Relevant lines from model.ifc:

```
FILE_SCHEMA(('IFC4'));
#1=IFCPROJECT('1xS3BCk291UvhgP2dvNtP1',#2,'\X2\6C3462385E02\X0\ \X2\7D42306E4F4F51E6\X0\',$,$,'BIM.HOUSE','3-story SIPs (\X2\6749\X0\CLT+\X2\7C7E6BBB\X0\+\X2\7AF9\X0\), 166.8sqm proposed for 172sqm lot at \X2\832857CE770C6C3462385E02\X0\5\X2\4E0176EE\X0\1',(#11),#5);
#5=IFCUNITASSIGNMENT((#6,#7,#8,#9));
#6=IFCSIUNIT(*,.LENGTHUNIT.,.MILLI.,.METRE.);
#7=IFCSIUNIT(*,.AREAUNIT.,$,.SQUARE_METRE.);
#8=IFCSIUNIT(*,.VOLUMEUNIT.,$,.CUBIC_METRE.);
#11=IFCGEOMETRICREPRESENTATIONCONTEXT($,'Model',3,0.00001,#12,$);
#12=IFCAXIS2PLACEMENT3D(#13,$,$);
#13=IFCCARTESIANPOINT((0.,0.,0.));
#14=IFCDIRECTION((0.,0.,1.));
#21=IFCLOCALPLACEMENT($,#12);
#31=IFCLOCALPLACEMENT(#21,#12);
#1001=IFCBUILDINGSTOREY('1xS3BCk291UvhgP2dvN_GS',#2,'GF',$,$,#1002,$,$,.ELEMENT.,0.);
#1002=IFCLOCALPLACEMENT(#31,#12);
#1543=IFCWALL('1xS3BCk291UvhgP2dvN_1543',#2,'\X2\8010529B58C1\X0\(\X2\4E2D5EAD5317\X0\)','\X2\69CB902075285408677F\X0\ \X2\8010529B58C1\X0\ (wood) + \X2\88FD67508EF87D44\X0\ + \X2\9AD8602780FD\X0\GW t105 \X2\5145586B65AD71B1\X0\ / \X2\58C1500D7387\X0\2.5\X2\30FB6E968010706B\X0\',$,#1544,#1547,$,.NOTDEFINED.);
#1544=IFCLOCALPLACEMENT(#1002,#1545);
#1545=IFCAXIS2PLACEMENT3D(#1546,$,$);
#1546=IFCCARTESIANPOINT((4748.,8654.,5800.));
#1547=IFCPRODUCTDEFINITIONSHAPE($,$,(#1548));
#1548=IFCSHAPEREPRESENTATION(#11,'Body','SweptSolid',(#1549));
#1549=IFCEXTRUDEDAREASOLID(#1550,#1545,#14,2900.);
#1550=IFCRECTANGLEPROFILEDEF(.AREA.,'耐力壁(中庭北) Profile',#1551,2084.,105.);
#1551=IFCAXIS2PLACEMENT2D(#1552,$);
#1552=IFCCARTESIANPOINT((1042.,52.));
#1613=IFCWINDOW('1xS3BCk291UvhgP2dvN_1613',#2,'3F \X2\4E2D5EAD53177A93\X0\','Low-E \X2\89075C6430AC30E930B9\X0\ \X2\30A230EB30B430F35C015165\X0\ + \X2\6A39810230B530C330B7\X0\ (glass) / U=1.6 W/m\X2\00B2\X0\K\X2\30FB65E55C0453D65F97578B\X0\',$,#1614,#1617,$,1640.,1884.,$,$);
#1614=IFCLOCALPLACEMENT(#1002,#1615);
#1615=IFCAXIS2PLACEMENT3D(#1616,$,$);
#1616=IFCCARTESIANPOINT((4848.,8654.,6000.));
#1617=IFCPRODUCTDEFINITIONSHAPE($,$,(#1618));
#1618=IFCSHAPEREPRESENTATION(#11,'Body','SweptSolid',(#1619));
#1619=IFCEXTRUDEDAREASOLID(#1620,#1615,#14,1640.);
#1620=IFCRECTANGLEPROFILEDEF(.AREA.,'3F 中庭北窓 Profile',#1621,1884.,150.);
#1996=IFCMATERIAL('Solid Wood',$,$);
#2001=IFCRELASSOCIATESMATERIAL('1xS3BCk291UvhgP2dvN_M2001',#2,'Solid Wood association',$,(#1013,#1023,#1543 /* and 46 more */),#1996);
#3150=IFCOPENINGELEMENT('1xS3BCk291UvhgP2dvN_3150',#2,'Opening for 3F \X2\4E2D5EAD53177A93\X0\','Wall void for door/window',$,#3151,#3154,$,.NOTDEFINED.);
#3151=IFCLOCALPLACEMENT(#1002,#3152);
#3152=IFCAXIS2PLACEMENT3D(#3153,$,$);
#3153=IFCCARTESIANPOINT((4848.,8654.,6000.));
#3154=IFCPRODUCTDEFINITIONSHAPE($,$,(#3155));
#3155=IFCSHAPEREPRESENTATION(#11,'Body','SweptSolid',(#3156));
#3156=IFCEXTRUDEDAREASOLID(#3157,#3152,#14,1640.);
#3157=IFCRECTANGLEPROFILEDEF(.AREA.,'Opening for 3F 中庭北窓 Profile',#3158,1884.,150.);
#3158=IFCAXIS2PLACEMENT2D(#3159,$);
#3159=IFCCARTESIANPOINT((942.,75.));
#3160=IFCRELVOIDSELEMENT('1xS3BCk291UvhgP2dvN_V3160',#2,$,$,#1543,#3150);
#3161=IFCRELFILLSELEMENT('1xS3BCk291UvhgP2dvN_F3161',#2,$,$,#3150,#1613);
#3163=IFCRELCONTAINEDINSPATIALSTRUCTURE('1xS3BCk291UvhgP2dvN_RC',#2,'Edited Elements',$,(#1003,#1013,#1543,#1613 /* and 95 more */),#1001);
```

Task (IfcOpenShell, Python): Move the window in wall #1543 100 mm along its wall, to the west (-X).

```python
import ifcopenshell
import ifcopenshell.api.geometry
import ifcopenshell.util.placement

model = ifcopenshell.open("model.ifc")

window = model.by_guid("1xS3BCk291UvhgP2dvN_1613")
opening = window.FillsVoids[0].RelatingOpeningElement
wall = opening.VoidsElements[0].RelatingBuildingElement

wall_matrix = ifcopenshell.util.placement.get_local_placement(wall.ObjectPlacement)
shift = wall_matrix[:3, 0] * -100.0
before = ifcopenshell.util.placement.get_local_placement(window.ObjectPlacement)[:3, 3].copy()

# The window is not placed relative to its opening, so move both.
for product in (opening, window):
    matrix = ifcopenshell.util.placement.get_local_placement(product.ObjectPlacement)
    matrix[:3, 3] += shift
    ifcopenshell.api.geometry.edit_object_placement(model, product=product, matrix=matrix, is_si=False)

after = ifcopenshell.util.placement.get_local_placement(window.ObjectPlacement)[:3, 3]
print("window moved by", (after - before).round(3) + 0.0)

model.write("model_rev.ifc")
```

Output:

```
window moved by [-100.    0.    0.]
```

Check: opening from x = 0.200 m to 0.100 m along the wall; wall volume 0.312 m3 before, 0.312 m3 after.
